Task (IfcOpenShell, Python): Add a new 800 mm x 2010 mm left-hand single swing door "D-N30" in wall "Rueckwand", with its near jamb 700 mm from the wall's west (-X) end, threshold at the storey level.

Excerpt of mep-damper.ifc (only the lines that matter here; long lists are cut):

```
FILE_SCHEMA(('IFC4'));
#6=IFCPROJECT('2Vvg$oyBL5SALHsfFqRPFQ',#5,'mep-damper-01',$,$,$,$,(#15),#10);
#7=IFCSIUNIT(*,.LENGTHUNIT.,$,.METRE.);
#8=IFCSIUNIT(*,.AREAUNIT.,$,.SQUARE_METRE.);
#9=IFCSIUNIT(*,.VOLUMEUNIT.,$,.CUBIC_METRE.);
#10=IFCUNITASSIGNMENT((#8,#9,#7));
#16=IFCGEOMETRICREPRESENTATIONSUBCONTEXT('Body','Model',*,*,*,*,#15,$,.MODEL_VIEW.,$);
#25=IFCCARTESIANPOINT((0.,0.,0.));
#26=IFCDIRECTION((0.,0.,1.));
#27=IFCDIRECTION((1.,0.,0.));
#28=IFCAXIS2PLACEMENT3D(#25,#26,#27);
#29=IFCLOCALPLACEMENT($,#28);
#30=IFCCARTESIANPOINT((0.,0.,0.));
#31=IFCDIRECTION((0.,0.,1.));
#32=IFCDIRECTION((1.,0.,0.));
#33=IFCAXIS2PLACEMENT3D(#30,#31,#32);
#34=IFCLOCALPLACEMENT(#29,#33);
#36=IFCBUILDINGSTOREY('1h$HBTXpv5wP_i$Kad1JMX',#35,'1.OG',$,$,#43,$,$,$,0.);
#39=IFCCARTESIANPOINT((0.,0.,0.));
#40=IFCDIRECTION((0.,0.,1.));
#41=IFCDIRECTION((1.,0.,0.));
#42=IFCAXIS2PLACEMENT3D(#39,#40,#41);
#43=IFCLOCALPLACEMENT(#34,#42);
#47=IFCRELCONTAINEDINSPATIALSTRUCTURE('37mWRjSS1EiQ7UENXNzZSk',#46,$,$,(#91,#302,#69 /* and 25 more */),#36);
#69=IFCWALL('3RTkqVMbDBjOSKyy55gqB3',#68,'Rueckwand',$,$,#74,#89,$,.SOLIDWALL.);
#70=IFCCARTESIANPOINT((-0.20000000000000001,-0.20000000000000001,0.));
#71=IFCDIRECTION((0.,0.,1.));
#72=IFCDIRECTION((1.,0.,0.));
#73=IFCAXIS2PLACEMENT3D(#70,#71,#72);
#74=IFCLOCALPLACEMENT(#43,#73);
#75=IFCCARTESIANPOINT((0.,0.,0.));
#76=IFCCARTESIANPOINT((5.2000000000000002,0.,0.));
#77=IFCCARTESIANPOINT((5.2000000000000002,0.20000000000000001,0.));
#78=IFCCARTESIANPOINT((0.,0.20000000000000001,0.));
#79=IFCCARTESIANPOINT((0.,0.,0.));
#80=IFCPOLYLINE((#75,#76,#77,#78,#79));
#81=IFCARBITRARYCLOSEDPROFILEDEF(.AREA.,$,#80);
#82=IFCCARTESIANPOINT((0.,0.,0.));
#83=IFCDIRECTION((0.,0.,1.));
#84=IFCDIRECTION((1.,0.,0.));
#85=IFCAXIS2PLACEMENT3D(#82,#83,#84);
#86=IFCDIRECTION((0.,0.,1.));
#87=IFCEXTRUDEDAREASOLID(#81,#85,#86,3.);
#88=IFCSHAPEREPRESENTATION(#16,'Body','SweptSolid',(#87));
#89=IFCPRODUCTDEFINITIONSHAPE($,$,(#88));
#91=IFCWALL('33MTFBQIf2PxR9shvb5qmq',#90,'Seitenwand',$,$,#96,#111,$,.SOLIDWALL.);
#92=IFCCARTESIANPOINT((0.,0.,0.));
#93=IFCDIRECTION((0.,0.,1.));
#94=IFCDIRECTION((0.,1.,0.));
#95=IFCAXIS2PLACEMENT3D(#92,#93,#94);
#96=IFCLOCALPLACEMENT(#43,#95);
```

```python
import numpy as np
import ifcopenshell
import ifcopenshell.api.feature
import ifcopenshell.api.geometry
import ifcopenshell.api.root
import ifcopenshell.api.spatial
import ifcopenshell.geom
import ifcopenshell.util.element
import ifcopenshell.util.placement
import ifcopenshell.util.representation
import ifcopenshell.util.shape
import ifcopenshell.util.unit

model = ifcopenshell.open("mep-damper.ifc")
unit_scale = ifcopenshell.util.unit.calculate_unit_scale(model)
settings = ifcopenshell.geom.settings()


def volume(element):
    """Net volume in cubic metres, openings subtracted."""
    shape = ifcopenshell.geom.create_shape(settings, element)
    return ifcopenshell.util.shape.get_volume(shape.geometry)


wall = model.by_guid("3RTkqVMbDBjOSKyy55gqB3")
storey = ifcopenshell.util.element.get_container(wall, ifc_class="IfcBuildingStorey")
context = ifcopenshell.util.representation.get_context(model, "Model", "Body", "MODEL_VIEW")
before = volume(wall)

width, height, from_end, sill = 0.8, 2.01, 0.7, 0.0  # metres

# The wall runs along its own X axis, and the end named is its -X end.
wall_shape = ifcopenshell.geom.create_shape(settings, wall)
x, y, z = ifcopenshell.util.shape.get_vertices(wall_shape.geometry).T
start = x.min() + from_end
face, thickness = float(y.min()), float(y.max() - y.min())
wall_matrix = ifcopenshell.util.placement.get_local_placement(wall.ObjectPlacement)
level = ifcopenshell.util.placement.get_local_placement(storey.ObjectPlacement)[2, 3]


def in_wall(x, y):
    """Placement at x, y metres in the wall's axes, at sill height."""
    matrix = wall_matrix.copy()
    matrix[:, 3] = wall_matrix @ np.array([x / unit_scale, y / unit_scale, 0.0, 1.0])
    matrix[2, 3] = level + sill / unit_scale
    return matrix


# Opening: a box that overshoots both wall faces by 50 mm.
opening = ifcopenshell.api.root.create_entity(model, ifc_class="IfcOpeningElement", predefined_type="OPENING")
box = ifcopenshell.api.geometry.add_wall_representation(
    model, context=context, length=width, height=height, thickness=thickness + 0.1
)
ifcopenshell.api.geometry.assign_representation(model, product=opening, representation=box)
ifcopenshell.api.geometry.edit_object_placement(model, product=opening, matrix=in_wall(start, face - 0.05), is_si=False)
ifcopenshell.api.feature.add_feature(model, feature=opening, element=wall)

door = ifcopenshell.api.root.create_entity(model, ifc_class="IfcDoor", name="D-N30", predefined_type="DOOR")
door.OverallWidth, door.OverallHeight = width / unit_scale, height / unit_scale
door.OperationType = "SINGLE_SWING_LEFT"
body = ifcopenshell.api.geometry.add_door_representation(
    model,
    context=context,
    overall_width=door.OverallWidth,
    overall_height=door.OverallHeight,
    operation_type="SINGLE_SWING_LEFT",
    lining_properties={"LiningDepth": thickness / unit_scale, "ThresholdDepth": thickness / unit_scale},
)
ifcopenshell.api.geometry.assign_representation(model, product=door, representation=body)
ifcopenshell.api.spatial.assign_container(model, products=[door], relating_structure=storey)
ifcopenshell.api.feature.add_filling(model, opening=opening, element=door)

# The lining spans the wall, so the door starts at the wall face.
ifcopenshell.api.geometry.edit_object_placement(model, product=door, matrix=in_wall(start, face), is_si=False)

after = volume(wall)

print(f"wall volume {before:.3f} -> {after:.3f} m3")

model.write("mep-damper_updated.ifc")
```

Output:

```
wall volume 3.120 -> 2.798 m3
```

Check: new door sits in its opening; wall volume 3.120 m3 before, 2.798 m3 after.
